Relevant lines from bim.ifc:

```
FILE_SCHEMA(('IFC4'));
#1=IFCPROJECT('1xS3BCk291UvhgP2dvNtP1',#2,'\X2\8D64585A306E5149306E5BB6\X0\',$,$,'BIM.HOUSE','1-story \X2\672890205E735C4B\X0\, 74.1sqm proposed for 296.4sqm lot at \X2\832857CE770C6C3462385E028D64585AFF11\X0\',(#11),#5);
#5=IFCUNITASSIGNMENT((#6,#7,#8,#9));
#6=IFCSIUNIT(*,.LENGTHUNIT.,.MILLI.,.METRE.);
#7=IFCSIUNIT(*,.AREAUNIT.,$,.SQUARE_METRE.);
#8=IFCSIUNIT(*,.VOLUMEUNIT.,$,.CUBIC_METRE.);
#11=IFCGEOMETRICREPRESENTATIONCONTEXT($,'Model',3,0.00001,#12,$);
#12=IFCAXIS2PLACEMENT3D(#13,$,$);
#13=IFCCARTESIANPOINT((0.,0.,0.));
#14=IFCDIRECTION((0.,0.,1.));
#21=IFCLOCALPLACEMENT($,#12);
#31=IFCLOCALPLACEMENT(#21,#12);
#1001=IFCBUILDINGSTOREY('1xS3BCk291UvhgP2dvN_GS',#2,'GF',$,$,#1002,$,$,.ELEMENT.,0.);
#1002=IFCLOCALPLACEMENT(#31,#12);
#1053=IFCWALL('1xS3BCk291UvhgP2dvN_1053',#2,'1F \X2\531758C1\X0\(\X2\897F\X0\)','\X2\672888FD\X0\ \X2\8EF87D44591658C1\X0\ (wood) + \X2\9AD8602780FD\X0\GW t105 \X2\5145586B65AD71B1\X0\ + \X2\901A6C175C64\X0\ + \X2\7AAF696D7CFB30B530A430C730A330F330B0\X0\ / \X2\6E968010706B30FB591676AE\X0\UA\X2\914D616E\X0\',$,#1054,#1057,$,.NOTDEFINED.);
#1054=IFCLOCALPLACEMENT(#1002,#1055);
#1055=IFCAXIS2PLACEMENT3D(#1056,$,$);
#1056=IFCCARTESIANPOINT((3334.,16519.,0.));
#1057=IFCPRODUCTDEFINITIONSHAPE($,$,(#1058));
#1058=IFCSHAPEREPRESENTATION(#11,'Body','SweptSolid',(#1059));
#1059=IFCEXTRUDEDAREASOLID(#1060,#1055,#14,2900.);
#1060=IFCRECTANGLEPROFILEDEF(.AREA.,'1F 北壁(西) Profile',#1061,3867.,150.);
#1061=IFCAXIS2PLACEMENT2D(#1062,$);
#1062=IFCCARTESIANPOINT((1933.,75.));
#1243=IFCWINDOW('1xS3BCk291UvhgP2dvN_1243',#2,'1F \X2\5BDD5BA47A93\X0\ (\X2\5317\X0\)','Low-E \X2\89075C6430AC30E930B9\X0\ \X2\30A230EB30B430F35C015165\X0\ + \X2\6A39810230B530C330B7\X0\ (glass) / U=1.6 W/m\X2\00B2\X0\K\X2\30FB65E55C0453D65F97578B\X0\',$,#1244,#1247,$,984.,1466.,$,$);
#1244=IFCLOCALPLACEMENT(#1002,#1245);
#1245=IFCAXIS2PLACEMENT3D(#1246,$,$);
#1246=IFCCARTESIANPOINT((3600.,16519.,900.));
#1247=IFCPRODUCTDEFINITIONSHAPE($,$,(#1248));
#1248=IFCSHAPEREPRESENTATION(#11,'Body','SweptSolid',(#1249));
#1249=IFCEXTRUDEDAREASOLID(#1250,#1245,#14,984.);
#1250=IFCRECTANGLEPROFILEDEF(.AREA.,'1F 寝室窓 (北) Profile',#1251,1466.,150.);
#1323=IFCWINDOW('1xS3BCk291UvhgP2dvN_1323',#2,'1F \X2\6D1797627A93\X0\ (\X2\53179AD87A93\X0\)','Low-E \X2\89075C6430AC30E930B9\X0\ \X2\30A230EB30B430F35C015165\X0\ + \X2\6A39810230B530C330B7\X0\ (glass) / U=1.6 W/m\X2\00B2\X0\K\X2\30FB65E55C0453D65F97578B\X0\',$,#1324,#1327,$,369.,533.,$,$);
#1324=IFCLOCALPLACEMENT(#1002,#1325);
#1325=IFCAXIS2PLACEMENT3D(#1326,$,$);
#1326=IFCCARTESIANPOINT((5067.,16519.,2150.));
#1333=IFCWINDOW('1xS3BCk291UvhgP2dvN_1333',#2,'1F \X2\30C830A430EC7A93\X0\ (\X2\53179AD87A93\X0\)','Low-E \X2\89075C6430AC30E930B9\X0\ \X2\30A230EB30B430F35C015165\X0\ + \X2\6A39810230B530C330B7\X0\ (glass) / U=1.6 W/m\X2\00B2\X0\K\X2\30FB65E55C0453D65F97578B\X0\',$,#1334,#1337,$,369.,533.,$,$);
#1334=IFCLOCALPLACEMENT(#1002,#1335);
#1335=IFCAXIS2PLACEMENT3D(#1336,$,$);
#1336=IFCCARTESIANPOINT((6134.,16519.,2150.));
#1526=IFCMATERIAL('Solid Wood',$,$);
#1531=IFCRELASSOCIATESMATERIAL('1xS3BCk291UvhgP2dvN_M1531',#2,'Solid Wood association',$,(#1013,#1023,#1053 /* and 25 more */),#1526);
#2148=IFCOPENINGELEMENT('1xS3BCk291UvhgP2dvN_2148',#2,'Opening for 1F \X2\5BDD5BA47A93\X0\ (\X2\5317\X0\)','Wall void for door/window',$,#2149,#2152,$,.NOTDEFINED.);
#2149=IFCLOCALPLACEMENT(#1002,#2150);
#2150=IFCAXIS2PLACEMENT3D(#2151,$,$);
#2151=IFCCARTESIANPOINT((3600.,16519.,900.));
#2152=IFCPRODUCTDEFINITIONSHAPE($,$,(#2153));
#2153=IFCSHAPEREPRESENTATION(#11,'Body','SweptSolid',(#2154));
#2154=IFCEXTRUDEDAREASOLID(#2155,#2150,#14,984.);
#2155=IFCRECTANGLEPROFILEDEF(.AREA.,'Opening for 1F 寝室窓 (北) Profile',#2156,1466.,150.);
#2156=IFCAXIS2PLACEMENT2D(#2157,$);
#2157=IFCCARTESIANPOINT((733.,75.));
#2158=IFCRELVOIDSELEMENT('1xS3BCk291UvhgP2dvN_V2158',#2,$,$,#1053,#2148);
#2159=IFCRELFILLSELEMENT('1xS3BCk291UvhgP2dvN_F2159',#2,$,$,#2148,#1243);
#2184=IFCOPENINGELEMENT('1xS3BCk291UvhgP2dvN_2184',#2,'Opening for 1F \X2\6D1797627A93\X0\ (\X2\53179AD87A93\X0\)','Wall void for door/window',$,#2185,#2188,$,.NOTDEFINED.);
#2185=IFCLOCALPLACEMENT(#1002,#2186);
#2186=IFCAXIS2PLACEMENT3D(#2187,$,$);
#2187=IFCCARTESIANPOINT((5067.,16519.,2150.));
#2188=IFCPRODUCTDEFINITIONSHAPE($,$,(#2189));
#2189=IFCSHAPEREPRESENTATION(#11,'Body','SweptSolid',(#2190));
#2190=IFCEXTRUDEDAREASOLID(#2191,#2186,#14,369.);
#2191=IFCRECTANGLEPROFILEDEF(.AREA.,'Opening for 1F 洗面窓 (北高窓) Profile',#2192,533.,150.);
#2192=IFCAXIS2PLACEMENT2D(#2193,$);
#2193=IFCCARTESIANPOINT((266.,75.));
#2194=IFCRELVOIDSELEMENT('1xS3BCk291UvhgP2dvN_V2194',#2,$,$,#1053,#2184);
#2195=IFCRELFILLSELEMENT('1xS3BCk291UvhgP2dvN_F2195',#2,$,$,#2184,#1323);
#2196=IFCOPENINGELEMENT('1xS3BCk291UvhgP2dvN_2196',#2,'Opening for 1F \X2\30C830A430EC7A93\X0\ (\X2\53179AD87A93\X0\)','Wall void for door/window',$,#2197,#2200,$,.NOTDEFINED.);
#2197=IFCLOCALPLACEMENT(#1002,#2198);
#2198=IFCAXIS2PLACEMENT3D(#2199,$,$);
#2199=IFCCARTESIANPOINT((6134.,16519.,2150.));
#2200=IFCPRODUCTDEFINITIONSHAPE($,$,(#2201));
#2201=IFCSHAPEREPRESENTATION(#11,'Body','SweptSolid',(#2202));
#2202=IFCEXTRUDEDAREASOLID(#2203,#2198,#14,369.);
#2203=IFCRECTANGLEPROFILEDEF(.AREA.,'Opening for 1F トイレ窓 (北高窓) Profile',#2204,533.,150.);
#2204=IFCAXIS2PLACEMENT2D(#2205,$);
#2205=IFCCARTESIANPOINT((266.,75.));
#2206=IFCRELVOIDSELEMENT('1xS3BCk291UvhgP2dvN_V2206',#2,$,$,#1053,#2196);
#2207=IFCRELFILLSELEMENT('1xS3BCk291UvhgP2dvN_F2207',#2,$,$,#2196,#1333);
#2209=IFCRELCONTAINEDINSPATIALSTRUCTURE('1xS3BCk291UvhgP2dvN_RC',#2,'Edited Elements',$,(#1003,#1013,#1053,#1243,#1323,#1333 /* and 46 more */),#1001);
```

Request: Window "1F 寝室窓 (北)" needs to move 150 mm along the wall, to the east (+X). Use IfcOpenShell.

```python
import ifcopenshell
import ifcopenshell.api.geometry
import ifcopenshell.util.placement
import ifcopenshell.util.unit

model = ifcopenshell.open("bim.ifc")
unit_scale = ifcopenshell.util.unit.calculate_unit_scale(model)

window = model.by_id(1243)
opening = window.FillsVoids[0].RelatingOpeningElement
wall = opening.VoidsElements[0].RelatingBuildingElement

wall_matrix = ifcopenshell.util.placement.get_local_placement(wall.ObjectPlacement)
shift = wall_matrix[:3, 0] * 0.15 / unit_scale
before = ifcopenshell.util.placement.get_local_placement(window.ObjectPlacement)[:3, 3].copy()

# The window is not placed relative to its opening, so move both.
for product in (opening, window):
    matrix = ifcopenshell.util.placement.get_local_placement(product.ObjectPlacement)
    matrix[:3, 3] += shift
    ifcopenshell.api.geometry.edit_object_placement(model, product=product, matrix=matrix, is_si=False)

after = ifcopenshell.util.placement.get_local_placement(window.ObjectPlacement)[:3, 3]
print("window moved by", (after - before).round(3) + 0.0)

model.write("bim-out.ifc")
```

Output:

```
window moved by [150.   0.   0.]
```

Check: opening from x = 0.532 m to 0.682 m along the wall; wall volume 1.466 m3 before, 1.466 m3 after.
